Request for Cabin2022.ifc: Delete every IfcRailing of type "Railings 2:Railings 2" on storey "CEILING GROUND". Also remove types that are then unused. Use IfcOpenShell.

First a look at what the model holds.

```python
import ifcopenshell
import ifcopenshell.util.element

model = ifcopenshell.open("Cabin2022.ifc")
print(model.schema)
storey = next(s for s in model.by_type("IfcBuildingStorey") if s.Name == "CEILING GROUND")
railings = [e for e in ifcopenshell.util.element.get_decomposition(storey) if e.is_a("IfcRailing")]
seen = {}
for e in railings:
    element_type = ifcopenshell.util.element.get_type(e)
    name = element_type.Name if element_type not in (None, e) else None
    seen[name] = seen.get(name, 0) + 1
for name, count in sorted(seen.items(), key=str):
    print(count, "x", name)
```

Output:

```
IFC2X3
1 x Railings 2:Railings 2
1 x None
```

```python
import ifcopenshell
import ifcopenshell.api.root
import ifcopenshell.util.element

model = ifcopenshell.open("Cabin2022.ifc")

storey = next(s for s in model.by_type("IfcBuildingStorey") if s.Name == "CEILING GROUND")
railings = [e for e in ifcopenshell.util.element.get_decomposition(storey) if e.is_a("IfcRailing")]
targets = [e for e in railings if (t := ifcopenshell.util.element.get_type(e)) not in (None, e) and t.Name == "Railings 2:Railings 2"]
types = {ifcopenshell.util.element.get_type(e) for e in targets} - {None, *targets}

for e in targets:
    ifcopenshell.api.root.remove_product(model, product=e)
print(len(targets), "removed")

unused = [t for t in types if not ifcopenshell.util.element.get_types(t)]
for t in unused:
    ifcopenshell.api.root.remove_product(model, product=t)
print(len(unused), "unused types removed")

model.write("Cabin2022_updated.ifc")
```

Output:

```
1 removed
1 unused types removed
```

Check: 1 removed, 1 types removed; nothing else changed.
